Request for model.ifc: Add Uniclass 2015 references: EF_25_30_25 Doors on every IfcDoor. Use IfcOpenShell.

First a look at what the model holds.

```python
import ifcopenshell

model = ifcopenshell.open("model.ifc")
print(model.schema)
print("classifications:", [c.Name for c in model.by_type("IfcClassification")])
for ifc_class in ("IfcDoor", "IfcRoof", "IfcStair", "IfcWall", "IfcWindow"):
    print(ifc_class, len(model.by_type(ifc_class)))
```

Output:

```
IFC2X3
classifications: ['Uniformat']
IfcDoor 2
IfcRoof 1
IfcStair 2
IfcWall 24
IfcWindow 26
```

```python
import ifcopenshell
import ifcopenshell.api.classification

model = ifcopenshell.open("model.ifc")

# IFC2X3 requires Source and Edition and has no link from the project to the system.
system = model.create_entity("IfcClassification", Source="NBS", Edition="2015", Name="Uniclass 2015")

codes = {
    "IfcDoor": ("EF_25_30_25", "Doors"),
}
for ifc_class, (code, name) in codes.items():
    products = model.by_type(ifc_class)
    ifcopenshell.api.classification.add_reference(
        model, products=products, classification=system, identification=code, name=name
    )
    print(code, len(products))

model.write("model_updated.ifc")
```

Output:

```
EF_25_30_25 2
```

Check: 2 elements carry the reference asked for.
